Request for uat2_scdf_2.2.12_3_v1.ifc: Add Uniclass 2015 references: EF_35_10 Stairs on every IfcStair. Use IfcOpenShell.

First a look at what the model holds.

```python
import ifcopenshell

model = ifcopenshell.open("uat2_scdf_2.2.12_3_v1.ifc")
print(model.schema)
print("classifications:", [c.Name for c in model.by_type("IfcClassification")])
for ifc_class in ("IfcDoor", "IfcRoof", "IfcStair", "IfcWall", "IfcWindow"):
    print(ifc_class, len(model.by_type(ifc_class)))
```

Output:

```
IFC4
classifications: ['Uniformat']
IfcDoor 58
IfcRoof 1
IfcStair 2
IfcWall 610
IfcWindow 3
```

```python
import ifcopenshell
import ifcopenshell.api.classification

model = ifcopenshell.open("uat2_scdf_2.2.12_3_v1.ifc")

system = ifcopenshell.api.classification.add_classification(model, classification="Uniclass 2015")

codes = {
    "IfcStair": ("EF_35_10", "Stairs"),
}
for ifc_class, (code, name) in codes.items():
    products = model.by_type(ifc_class)
    ifcopenshell.api.classification.add_reference(
        model, products=products, classification=system, identification=code, name=name
    )
    print(code, len(products))

model.write("uat2_scdf_2.2.12_3_v1_updated.ifc")
```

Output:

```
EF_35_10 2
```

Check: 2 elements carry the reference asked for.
